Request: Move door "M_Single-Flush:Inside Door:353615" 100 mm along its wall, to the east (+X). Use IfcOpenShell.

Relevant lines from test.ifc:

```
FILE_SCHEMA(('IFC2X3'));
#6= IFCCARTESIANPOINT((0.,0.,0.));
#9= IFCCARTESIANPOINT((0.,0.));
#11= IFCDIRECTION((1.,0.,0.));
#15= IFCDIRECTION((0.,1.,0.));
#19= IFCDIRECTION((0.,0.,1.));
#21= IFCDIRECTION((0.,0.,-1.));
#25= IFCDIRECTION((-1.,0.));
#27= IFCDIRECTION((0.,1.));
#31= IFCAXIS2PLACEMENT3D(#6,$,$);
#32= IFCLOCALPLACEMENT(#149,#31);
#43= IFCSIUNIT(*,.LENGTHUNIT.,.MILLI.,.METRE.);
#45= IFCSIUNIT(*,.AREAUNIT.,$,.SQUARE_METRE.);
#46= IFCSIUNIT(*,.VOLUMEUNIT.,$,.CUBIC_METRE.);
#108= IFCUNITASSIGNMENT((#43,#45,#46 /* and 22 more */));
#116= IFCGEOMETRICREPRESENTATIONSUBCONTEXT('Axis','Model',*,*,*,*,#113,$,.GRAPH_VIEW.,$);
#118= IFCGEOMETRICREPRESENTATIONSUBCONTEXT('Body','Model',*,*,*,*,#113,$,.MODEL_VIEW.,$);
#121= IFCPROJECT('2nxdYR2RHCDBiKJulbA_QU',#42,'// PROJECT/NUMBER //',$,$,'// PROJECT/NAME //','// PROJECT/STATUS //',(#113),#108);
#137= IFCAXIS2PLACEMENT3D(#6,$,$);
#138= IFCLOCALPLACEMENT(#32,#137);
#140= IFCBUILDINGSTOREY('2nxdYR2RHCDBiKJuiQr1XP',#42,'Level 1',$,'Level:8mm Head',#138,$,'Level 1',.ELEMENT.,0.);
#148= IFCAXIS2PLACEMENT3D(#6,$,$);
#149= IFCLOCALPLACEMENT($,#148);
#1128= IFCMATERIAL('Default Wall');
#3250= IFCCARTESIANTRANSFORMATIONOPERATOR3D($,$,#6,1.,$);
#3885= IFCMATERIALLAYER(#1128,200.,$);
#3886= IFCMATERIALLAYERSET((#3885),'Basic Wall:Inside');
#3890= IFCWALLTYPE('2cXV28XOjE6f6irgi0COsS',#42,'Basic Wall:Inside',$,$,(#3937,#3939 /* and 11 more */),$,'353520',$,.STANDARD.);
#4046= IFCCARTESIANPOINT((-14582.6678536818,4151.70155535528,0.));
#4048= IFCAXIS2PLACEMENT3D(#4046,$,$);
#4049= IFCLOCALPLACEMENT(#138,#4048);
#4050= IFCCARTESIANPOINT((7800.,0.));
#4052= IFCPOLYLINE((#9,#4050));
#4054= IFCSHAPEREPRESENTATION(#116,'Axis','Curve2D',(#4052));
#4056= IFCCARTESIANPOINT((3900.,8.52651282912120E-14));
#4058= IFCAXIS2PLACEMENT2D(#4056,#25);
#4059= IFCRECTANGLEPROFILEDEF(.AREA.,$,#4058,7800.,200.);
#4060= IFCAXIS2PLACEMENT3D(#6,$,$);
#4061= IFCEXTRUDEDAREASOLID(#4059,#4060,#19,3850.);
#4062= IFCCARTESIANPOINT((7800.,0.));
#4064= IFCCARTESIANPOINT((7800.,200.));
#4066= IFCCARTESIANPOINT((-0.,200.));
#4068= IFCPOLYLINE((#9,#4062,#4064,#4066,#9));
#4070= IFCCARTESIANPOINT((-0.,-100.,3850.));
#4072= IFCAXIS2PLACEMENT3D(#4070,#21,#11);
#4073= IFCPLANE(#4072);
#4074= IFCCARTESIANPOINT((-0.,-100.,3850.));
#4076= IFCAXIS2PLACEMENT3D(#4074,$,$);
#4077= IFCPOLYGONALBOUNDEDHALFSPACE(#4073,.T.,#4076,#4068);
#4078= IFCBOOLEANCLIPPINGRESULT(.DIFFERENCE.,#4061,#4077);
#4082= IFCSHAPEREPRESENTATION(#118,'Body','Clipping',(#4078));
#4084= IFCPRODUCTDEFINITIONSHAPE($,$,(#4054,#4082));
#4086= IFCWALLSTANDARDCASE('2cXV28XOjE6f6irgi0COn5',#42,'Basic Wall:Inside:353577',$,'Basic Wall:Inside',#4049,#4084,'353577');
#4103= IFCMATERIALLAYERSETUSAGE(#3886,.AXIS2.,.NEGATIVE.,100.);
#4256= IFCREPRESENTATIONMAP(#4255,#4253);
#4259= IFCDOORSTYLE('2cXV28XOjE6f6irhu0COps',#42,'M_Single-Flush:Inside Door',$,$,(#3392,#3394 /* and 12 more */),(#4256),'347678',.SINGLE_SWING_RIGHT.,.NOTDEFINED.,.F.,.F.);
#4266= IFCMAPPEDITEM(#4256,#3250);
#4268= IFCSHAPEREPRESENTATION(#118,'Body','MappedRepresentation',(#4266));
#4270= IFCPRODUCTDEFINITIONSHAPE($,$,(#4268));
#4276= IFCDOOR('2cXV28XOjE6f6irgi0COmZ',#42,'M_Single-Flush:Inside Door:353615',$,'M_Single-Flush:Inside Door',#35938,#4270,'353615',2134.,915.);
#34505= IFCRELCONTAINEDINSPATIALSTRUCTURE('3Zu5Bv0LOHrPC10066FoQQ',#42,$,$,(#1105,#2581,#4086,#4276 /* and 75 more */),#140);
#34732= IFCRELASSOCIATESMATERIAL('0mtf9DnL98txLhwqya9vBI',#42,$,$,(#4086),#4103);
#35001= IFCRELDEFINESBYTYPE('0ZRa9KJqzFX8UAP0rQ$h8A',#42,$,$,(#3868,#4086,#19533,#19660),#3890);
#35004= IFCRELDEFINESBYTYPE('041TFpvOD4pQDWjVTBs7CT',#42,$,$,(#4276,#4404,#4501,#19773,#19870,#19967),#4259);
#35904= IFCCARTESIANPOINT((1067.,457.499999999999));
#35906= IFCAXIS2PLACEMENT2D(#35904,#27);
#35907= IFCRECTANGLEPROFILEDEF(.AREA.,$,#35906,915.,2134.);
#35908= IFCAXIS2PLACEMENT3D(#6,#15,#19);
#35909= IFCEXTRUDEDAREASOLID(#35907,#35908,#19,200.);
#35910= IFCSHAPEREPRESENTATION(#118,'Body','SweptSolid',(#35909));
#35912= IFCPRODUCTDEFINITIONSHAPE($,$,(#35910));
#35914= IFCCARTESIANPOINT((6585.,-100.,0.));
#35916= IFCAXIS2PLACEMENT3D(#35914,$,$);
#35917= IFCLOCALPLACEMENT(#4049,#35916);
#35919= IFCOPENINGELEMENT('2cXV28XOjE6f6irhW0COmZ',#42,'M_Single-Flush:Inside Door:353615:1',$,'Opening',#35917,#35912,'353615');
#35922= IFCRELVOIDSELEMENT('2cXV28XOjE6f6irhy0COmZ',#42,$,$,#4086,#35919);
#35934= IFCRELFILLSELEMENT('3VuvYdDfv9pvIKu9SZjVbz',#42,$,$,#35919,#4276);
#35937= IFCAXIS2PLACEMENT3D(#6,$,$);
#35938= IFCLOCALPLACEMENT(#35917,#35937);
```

```python
import ifcopenshell
import ifcopenshell.api.geometry
import ifcopenshell.util.placement

model = ifcopenshell.open("test.ifc")

door = model.by_guid("2cXV28XOjE6f6irgi0COmZ")
opening = door.FillsVoids[0].RelatingOpeningElement
wall = opening.VoidsElements[0].RelatingBuildingElement

wall_matrix = ifcopenshell.util.placement.get_local_placement(wall.ObjectPlacement)
shift = wall_matrix[:3, 0] * 100.0
before = ifcopenshell.util.placement.get_local_placement(door.ObjectPlacement)[:3, 3].copy()

# The door is placed relative to its opening, so it follows when the opening moves.
matrix = ifcopenshell.util.placement.get_local_placement(opening.ObjectPlacement)
matrix[:3, 3] += shift
ifcopenshell.api.geometry.edit_object_placement(
    model, product=opening, matrix=matrix, is_si=False, should_transform_children=True
)

after = ifcopenshell.util.placement.get_local_placement(door.ObjectPlacement)[:3, 3]
print("door moved by", (after - before).round(3) + 0.0)

model.write("test_v2.ifc")
```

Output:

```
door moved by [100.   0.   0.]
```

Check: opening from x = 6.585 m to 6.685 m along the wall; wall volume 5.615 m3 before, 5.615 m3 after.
